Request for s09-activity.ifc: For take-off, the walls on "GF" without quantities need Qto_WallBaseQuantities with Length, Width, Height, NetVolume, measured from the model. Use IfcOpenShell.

First a look at what the model holds.

```python
import ifcopenshell
import ifcopenshell.util.element
import ifcopenshell.util.unit

model = ifcopenshell.open("s09-activity.ifc")
print(model.schema)
for unit_type in ("LENGTHUNIT", "AREAUNIT", "VOLUMEUNIT"):
    print(unit_type, ifcopenshell.util.unit.calculate_unit_scale(model, unit_type))
storey = next(s for s in model.by_type("IfcBuildingStorey") if s.Name == "GF")
walls = [e for e in ifcopenshell.util.element.get_decomposition(storey) if e.is_a("IfcWall")]
for e in sorted(walls, key=lambda e: e.id()):
    print(e.id(), e.is_a(), e.Name, list(ifcopenshell.util.element.get_psets(e, qtos_only=True)), sep=" | ")
```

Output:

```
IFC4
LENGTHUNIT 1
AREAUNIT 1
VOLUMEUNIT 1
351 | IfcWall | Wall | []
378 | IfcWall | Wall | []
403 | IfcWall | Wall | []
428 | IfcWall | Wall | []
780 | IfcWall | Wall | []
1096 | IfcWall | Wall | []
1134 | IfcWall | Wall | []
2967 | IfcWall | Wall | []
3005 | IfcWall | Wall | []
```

```python
import ifcopenshell
import ifcopenshell.api.pset
import ifcopenshell.geom
import ifcopenshell.util.element
import ifcopenshell.util.shape
import ifcopenshell.util.unit

model = ifcopenshell.open("s09-activity.ifc")
unit_scale = ifcopenshell.util.unit.calculate_unit_scale(model)
volume_scale = ifcopenshell.util.unit.calculate_unit_scale(model, "VOLUMEUNIT")
settings = ifcopenshell.geom.settings()

storey = next(s for s in model.by_type("IfcBuildingStorey") if s.Name == "GF")
walls = [e for e in ifcopenshell.util.element.get_decomposition(storey) if e.is_a("IfcWall")]

for e in sorted(walls, key=lambda e: e.id()):
    if ifcopenshell.util.element.get_psets(e, qtos_only=True, should_inherit=False):
        continue
    # Geometry comes back in metres, in the element's own axes.
    shape = ifcopenshell.geom.create_shape(settings, e)
    values = {
        "Length": ifcopenshell.util.shape.get_x(shape.geometry) / unit_scale,
        "Width": ifcopenshell.util.shape.get_y(shape.geometry) / unit_scale,
        "Height": ifcopenshell.util.shape.get_z(shape.geometry) / unit_scale,
        "NetVolume": ifcopenshell.util.shape.get_volume(shape.geometry) / volume_scale,
    }
    qto = ifcopenshell.api.pset.add_qto(model, product=e, name="Qto_WallBaseQuantities")
    ifcopenshell.api.pset.edit_qto(model, qto=qto, properties=values)
    print(e.id(), {k: round(v, 3) for k, v in values.items()})

model.write("s09-activity_rev.ifc")
```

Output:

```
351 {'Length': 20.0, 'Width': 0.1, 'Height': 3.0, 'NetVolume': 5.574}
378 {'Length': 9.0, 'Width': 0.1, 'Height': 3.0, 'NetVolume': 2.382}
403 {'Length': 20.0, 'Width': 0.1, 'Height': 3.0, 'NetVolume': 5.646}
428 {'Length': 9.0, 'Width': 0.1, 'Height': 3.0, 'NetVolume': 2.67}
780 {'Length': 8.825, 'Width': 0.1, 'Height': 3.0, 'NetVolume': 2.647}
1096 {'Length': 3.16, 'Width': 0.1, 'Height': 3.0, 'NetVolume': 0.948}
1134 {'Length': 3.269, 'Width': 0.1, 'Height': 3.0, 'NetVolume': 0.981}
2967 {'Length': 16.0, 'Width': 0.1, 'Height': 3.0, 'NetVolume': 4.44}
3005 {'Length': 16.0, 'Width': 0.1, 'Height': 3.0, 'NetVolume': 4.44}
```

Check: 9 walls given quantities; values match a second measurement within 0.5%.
